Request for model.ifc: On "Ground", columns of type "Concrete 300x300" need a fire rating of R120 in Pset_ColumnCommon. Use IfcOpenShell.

First a look at what the model holds.

```python
import ifcopenshell
import ifcopenshell.util.element

model = ifcopenshell.open("model.ifc")
print(model.schema)
storey = next(s for s in model.by_type("IfcBuildingStorey") if s.Name == "Ground")
columns = [e for e in ifcopenshell.util.element.get_decomposition(storey) if e.is_a("IfcColumn")]
seen = {}
for e in columns:
    element_type = ifcopenshell.util.element.get_type(e)
    key = (element_type.Name if element_type != e and element_type else None, ifcopenshell.util.element.get_pset(e, "Pset_ColumnCommon", "FireRating"))
    seen[key] = seen.get(key, 0) + 1
for (name, value), count in sorted(seen.items(), key=str):
    print(count, "x", name, "|", value)
```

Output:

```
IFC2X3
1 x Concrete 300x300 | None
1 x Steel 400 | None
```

```python
import ifcopenshell
import ifcopenshell.api.pset
import ifcopenshell.util.element

model = ifcopenshell.open("model.ifc")

storey = next(s for s in model.by_type("IfcBuildingStorey") if s.Name == "Ground")
columns = [e for e in ifcopenshell.util.element.get_decomposition(storey) if e.is_a("IfcColumn")]

count = 0
for e in columns:
    element_type = ifcopenshell.util.element.get_type(e)
    if element_type in (None, e) or element_type.Name != "Concrete 300x300":
        continue
    # add_pset returns the element's existing set when there is one.
    pset = ifcopenshell.api.pset.add_pset(model, product=e, name="Pset_ColumnCommon")
    ifcopenshell.api.pset.edit_pset(model, pset=pset, properties={"FireRating": "R120"})
    count += 1

print(count, "columns updated")

model.write("model_edited.ifc")
```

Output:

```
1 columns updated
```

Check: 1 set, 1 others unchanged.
